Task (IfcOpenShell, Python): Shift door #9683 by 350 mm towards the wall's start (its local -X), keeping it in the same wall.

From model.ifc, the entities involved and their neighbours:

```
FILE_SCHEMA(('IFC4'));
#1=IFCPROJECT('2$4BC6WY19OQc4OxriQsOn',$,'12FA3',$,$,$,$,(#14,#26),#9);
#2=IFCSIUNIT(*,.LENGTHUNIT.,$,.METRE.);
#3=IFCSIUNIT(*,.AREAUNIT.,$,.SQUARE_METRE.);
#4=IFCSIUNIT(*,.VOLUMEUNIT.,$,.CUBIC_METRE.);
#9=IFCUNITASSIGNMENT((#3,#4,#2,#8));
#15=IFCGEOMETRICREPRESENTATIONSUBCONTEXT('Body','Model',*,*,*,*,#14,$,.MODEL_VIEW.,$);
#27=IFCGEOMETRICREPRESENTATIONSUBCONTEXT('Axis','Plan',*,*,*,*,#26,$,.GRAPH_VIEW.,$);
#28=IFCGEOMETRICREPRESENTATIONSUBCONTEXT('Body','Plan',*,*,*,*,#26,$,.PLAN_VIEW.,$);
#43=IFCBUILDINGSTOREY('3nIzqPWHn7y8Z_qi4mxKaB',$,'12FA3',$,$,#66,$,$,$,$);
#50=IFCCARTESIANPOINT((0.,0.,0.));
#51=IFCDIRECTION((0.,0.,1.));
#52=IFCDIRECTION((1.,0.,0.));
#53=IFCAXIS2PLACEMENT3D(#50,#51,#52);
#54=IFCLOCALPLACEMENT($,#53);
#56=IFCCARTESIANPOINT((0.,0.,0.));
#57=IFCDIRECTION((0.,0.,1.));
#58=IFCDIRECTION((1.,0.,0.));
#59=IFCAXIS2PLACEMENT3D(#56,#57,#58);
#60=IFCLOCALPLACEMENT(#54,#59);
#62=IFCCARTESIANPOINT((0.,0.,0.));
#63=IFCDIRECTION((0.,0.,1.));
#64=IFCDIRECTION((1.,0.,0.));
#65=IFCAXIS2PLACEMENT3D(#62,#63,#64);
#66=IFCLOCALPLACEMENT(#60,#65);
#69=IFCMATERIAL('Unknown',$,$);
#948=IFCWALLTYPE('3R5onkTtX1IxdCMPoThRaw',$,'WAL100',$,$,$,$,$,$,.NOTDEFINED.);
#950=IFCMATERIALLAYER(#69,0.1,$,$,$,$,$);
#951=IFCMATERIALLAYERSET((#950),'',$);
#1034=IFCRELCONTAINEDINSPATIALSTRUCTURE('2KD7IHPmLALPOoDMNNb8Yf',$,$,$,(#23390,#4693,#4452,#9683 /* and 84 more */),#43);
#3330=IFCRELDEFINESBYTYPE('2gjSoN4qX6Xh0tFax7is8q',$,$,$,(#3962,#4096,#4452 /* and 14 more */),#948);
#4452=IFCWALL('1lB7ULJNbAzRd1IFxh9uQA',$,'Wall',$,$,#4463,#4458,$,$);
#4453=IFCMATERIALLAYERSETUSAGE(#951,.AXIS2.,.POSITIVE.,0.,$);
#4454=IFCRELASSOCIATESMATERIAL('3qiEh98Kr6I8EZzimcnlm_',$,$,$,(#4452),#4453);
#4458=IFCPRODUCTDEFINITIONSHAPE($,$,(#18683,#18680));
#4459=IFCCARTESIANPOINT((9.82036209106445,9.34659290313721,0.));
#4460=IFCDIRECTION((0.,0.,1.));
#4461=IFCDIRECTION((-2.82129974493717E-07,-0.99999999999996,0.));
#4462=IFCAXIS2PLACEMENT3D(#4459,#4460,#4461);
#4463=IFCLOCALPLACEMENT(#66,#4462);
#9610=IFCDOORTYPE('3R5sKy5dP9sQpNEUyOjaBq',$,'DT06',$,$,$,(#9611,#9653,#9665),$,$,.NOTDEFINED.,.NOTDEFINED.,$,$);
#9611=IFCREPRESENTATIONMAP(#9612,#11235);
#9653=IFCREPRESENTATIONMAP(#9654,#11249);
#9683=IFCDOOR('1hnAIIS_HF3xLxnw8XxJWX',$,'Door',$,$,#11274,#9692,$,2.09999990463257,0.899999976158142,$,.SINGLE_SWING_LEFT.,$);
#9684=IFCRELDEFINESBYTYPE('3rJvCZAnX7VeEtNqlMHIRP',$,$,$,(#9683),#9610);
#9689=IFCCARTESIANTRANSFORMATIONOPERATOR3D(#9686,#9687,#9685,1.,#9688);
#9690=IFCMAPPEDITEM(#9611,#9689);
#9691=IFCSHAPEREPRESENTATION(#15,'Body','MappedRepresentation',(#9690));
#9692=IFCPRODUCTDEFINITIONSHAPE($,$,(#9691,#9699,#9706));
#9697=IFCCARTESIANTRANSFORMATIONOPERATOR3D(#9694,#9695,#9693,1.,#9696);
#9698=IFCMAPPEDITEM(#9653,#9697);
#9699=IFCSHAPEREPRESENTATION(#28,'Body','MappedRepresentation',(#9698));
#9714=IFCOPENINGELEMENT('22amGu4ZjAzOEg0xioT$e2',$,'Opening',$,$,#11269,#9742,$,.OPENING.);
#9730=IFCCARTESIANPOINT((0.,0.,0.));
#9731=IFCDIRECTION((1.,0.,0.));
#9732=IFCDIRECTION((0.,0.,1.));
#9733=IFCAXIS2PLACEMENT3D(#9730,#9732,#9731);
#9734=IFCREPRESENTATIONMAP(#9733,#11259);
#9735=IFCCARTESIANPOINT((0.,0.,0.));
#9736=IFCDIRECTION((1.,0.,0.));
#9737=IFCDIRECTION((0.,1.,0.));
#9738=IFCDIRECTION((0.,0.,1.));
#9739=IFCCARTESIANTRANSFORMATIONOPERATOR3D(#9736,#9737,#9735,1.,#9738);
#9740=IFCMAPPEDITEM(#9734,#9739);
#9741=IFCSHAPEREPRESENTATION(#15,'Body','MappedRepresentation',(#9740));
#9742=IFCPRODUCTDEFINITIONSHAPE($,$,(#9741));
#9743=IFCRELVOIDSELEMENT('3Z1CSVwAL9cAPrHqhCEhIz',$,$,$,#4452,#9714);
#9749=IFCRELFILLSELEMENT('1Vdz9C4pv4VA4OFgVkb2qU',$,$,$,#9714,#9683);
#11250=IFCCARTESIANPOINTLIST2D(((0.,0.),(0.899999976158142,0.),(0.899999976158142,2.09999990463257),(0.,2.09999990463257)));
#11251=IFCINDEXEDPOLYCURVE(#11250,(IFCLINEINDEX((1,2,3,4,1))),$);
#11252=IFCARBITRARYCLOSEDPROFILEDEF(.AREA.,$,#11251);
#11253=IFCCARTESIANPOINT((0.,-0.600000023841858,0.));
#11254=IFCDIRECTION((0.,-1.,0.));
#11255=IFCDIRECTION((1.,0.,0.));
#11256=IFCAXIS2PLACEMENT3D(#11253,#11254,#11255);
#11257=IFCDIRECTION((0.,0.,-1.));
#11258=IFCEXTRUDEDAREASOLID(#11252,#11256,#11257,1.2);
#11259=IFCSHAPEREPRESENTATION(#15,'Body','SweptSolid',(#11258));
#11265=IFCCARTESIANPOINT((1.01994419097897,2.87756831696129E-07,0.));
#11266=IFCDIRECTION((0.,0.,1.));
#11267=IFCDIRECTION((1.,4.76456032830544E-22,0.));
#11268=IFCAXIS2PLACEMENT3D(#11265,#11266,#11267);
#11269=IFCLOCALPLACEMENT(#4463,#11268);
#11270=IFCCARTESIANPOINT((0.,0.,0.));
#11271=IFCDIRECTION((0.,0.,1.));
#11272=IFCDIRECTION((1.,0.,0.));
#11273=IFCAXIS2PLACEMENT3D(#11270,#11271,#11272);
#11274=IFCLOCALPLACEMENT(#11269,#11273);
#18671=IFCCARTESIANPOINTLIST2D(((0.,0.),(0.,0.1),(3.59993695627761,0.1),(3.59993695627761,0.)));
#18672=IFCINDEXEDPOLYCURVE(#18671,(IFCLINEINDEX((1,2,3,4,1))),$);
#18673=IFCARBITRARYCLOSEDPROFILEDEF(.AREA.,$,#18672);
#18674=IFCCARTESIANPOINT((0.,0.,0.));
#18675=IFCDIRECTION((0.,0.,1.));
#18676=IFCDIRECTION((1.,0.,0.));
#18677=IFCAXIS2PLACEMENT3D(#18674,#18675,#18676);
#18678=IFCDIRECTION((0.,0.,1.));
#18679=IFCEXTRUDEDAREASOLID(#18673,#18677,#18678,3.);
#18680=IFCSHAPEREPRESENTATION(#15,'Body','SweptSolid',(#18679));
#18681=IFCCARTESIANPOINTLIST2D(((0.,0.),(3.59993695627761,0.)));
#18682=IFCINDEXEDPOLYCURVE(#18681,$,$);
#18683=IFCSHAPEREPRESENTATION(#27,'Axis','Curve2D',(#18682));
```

```python
import ifcopenshell
import ifcopenshell.api.geometry
import ifcopenshell.util.placement

model = ifcopenshell.open("model.ifc")

door = model.by_guid("1hnAIIS_HF3xLxnw8XxJWX")
opening = door.FillsVoids[0].RelatingOpeningElement
wall = opening.VoidsElements[0].RelatingBuildingElement

wall_matrix = ifcopenshell.util.placement.get_local_placement(wall.ObjectPlacement)
shift = wall_matrix[:3, 0] * -0.35
before = ifcopenshell.util.placement.get_local_placement(door.ObjectPlacement)[:3, 3].copy()

# The door is placed relative to its opening, so it follows when the opening moves.
matrix = ifcopenshell.util.placement.get_local_placement(opening.ObjectPlacement)
matrix[:3, 3] += shift
ifcopenshell.api.geometry.edit_object_placement(
    model, product=opening, matrix=matrix, is_si=False, should_transform_children=True
)

after = ifcopenshell.util.placement.get_local_placement(door.ObjectPlacement)[:3, 3]
print("door moved by", (after - before).round(3) + 0.0)

model.write("model_updated.ifc")
```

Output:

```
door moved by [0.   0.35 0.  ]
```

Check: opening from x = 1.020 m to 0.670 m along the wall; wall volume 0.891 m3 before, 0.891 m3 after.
